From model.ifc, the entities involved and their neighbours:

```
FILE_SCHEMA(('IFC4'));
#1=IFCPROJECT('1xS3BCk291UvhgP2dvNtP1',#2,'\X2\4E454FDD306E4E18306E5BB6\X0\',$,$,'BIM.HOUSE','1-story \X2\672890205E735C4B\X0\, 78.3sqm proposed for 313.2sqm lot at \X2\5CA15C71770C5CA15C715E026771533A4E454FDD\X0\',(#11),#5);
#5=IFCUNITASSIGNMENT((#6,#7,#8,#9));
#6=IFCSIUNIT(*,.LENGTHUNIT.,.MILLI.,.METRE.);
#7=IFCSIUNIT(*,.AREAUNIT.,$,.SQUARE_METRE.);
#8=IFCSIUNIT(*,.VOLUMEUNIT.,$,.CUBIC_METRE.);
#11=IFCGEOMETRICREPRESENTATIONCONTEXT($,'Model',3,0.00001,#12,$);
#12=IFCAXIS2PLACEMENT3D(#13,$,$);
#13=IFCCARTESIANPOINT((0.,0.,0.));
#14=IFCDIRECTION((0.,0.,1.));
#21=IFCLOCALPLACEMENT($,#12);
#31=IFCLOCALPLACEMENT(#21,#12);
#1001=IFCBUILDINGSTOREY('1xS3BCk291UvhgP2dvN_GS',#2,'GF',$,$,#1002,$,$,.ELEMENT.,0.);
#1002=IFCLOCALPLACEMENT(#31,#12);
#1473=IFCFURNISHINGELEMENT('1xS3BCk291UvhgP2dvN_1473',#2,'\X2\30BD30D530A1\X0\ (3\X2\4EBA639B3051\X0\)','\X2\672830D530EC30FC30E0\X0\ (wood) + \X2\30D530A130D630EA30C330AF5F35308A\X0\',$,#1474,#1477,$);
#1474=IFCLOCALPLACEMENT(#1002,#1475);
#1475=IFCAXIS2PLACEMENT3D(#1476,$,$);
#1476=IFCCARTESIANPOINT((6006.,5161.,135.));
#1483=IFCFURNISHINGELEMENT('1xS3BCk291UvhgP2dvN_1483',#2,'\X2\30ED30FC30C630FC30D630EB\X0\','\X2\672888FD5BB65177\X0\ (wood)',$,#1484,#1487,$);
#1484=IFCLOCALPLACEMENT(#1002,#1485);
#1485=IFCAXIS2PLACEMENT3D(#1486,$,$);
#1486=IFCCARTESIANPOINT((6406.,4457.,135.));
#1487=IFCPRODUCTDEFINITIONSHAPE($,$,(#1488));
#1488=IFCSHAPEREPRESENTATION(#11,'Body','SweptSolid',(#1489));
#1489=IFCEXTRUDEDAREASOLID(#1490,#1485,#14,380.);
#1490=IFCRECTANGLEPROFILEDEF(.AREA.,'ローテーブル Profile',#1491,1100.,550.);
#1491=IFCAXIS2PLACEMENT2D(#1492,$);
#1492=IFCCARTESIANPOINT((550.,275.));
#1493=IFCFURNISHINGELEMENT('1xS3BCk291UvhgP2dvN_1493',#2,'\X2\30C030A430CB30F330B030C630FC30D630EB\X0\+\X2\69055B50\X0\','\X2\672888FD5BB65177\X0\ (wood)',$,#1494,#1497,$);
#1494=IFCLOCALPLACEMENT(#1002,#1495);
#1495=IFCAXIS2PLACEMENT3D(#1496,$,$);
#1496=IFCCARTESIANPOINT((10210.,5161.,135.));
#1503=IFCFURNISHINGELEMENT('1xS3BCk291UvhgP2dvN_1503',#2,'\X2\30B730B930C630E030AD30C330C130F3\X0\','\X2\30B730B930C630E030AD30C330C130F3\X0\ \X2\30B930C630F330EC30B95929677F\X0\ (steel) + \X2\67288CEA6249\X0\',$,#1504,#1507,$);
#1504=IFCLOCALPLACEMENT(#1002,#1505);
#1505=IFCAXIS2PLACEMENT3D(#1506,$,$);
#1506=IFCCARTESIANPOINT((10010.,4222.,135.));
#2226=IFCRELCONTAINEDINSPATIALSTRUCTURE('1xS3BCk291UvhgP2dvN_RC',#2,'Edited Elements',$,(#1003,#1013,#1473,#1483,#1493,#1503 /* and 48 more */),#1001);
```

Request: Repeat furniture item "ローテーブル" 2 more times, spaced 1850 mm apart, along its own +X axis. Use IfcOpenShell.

```python
import ifcopenshell
import ifcopenshell.api.geometry
import ifcopenshell.api.root
import ifcopenshell.util.element
import ifcopenshell.util.placement
import ifcopenshell.util.unit

model = ifcopenshell.open("model.ifc")
unit_scale = ifcopenshell.util.unit.calculate_unit_scale(model)


def reuse_history(source, copy):
    """copy_class also copies each property set's owner history, people and application; keep the originals."""
    for rel in copy.IsDefinedBy:
        if rel.is_a("IfcRelDefinesByProperties") and (history := rel.RelatingPropertyDefinition.OwnerHistory):
            rel.RelatingPropertyDefinition.OwnerHistory = source.OwnerHistory
            ifcopenshell.util.element.remove_deep2(model, history)


source = model.by_id(1483)
base = ifcopenshell.util.placement.get_local_placement(source.ObjectPlacement)
step = base[:3, 0] * 1.85 / unit_scale

for i in range(1, 3):
    copy = ifcopenshell.api.root.copy_class(model, product=source)
    copy.Representation = ifcopenshell.util.element.copy_deep(
        model, source.Representation, exclude=["IfcGeometricRepresentationContext", "IfcRepresentationMap"]
    )
    reuse_history(source, copy)
    matrix = base.copy()
    matrix[:3, 3] += i * step
    print("added at", matrix[:3, 3].round(3) + 0.0)
    ifcopenshell.api.geometry.edit_object_placement(model, product=copy, matrix=matrix, is_si=False)

model.write("model_rev.ifc")
```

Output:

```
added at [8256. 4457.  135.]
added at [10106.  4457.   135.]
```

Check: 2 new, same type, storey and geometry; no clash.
